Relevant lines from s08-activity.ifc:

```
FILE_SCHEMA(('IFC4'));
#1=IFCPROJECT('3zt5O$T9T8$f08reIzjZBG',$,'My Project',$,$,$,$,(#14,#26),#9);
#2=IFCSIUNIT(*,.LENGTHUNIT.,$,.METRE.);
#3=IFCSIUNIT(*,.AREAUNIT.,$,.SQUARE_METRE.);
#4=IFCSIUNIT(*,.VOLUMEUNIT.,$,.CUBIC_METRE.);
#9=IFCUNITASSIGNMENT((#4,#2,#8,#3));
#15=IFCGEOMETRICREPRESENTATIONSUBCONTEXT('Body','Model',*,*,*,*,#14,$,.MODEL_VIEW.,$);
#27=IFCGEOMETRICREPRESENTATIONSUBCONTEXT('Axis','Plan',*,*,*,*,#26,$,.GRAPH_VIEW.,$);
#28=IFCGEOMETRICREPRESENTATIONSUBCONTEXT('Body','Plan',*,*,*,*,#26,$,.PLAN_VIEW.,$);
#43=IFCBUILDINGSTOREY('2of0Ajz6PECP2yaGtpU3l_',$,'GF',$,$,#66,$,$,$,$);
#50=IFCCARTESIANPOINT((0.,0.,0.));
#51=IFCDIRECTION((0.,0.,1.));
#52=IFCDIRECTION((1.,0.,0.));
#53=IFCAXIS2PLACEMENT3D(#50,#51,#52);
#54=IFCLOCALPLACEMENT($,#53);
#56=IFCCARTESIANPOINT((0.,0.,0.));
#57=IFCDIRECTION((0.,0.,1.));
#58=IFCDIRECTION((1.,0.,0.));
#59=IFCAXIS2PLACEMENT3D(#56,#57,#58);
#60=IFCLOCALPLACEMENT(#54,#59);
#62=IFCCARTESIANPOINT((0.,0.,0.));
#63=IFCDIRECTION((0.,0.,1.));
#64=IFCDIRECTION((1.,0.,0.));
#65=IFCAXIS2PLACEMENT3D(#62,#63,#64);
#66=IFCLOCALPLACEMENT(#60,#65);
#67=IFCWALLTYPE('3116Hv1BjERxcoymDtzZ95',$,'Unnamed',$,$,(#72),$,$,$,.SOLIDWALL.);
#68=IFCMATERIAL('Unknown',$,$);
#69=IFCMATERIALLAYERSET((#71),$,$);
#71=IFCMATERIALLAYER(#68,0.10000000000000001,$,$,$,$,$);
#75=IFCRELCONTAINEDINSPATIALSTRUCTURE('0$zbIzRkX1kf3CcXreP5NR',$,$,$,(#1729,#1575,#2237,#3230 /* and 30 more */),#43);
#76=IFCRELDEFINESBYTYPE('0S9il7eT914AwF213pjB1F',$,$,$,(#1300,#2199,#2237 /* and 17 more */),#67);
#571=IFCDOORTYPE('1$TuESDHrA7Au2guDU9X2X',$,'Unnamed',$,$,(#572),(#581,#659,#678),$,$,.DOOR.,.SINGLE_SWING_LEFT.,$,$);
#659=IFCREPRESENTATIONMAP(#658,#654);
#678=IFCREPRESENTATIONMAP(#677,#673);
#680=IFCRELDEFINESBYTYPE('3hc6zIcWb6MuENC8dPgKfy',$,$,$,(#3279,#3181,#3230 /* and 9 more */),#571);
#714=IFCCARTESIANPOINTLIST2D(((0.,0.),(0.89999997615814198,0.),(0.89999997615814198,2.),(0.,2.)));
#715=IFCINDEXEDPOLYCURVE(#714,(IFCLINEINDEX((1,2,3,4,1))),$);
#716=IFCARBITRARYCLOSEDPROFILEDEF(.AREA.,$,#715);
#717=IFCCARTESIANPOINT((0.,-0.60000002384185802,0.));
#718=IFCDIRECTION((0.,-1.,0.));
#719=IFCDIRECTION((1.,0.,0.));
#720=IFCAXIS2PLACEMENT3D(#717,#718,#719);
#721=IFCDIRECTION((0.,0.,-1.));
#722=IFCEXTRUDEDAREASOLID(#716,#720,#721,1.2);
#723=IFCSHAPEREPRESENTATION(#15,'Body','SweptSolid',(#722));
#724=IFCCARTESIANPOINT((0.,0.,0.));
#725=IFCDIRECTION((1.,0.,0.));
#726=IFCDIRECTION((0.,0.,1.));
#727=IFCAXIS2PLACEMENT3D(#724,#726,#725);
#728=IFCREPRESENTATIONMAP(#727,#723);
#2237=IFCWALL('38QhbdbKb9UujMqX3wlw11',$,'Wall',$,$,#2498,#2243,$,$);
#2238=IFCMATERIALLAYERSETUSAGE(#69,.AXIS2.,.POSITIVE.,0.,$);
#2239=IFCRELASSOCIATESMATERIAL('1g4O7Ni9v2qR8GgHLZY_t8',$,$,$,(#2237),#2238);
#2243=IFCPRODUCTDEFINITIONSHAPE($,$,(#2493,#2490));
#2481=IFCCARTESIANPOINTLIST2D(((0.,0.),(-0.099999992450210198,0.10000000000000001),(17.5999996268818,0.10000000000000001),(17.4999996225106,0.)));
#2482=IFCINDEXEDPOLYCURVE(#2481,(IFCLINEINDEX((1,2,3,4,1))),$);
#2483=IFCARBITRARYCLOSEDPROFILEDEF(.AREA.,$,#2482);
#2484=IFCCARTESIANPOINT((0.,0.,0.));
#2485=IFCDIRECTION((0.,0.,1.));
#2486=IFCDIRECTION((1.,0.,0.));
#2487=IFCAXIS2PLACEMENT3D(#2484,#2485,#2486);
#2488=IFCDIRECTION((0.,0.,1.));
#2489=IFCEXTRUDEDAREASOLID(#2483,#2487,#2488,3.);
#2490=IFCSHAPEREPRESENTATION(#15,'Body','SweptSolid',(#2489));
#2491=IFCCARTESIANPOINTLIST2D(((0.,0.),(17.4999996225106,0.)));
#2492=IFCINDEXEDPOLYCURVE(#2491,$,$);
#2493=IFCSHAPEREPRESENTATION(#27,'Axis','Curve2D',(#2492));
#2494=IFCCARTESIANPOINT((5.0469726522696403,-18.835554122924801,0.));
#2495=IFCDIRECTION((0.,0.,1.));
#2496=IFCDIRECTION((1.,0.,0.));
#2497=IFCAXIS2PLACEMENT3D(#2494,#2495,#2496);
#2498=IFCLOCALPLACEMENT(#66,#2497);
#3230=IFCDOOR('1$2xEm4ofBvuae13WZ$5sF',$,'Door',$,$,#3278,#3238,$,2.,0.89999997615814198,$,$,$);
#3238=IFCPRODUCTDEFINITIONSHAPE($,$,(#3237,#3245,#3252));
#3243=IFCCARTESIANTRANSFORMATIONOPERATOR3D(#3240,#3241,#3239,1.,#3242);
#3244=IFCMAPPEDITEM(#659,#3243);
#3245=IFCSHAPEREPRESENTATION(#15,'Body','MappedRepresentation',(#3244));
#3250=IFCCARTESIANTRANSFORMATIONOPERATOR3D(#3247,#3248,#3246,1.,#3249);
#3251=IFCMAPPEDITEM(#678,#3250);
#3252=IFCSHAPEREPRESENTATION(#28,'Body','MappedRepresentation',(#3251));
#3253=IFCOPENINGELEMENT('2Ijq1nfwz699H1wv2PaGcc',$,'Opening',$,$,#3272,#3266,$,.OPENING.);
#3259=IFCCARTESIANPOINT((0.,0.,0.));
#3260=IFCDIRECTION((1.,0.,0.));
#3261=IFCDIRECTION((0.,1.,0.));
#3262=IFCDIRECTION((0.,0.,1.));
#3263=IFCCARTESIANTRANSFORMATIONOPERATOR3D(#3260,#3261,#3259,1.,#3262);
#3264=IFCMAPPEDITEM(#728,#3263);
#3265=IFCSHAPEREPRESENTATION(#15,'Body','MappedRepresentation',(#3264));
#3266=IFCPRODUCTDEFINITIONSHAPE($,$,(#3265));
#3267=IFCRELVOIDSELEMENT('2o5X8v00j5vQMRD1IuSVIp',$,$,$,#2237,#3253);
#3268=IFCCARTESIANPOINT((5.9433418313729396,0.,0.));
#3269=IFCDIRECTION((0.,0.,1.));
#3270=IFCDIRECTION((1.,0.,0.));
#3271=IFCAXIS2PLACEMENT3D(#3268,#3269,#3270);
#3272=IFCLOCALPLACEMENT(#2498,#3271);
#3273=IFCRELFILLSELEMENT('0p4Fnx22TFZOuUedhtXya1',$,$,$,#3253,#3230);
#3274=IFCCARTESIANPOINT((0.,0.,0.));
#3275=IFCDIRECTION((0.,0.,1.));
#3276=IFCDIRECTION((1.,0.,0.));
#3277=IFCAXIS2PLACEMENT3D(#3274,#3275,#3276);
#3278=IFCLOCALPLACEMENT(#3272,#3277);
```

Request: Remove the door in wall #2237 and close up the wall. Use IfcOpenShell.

```python
import ifcopenshell
import ifcopenshell.api.feature
import ifcopenshell.api.root
import ifcopenshell.geom
import ifcopenshell.util.shape

model = ifcopenshell.open("s08-activity.ifc")
settings = ifcopenshell.geom.settings()


def volume(element):
    """Net volume in cubic metres, openings subtracted."""
    shape = ifcopenshell.geom.create_shape(settings, element)
    return ifcopenshell.util.shape.get_volume(shape.geometry)


door = model.by_guid("1$2xEm4ofBvuae13WZ$5sF")
opening = door.FillsVoids[0].RelatingOpeningElement
wall = opening.VoidsElements[0].RelatingBuildingElement
before = volume(wall)

ifcopenshell.api.root.remove_product(model, product=door)
ifcopenshell.api.feature.remove_feature(model, feature=opening)

after = volume(wall)

print(f"wall volume {before:.3f} -> {after:.3f} m3")

model.write("s08-activity_v2.ifc")
```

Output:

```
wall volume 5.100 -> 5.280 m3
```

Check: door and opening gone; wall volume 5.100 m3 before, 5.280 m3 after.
